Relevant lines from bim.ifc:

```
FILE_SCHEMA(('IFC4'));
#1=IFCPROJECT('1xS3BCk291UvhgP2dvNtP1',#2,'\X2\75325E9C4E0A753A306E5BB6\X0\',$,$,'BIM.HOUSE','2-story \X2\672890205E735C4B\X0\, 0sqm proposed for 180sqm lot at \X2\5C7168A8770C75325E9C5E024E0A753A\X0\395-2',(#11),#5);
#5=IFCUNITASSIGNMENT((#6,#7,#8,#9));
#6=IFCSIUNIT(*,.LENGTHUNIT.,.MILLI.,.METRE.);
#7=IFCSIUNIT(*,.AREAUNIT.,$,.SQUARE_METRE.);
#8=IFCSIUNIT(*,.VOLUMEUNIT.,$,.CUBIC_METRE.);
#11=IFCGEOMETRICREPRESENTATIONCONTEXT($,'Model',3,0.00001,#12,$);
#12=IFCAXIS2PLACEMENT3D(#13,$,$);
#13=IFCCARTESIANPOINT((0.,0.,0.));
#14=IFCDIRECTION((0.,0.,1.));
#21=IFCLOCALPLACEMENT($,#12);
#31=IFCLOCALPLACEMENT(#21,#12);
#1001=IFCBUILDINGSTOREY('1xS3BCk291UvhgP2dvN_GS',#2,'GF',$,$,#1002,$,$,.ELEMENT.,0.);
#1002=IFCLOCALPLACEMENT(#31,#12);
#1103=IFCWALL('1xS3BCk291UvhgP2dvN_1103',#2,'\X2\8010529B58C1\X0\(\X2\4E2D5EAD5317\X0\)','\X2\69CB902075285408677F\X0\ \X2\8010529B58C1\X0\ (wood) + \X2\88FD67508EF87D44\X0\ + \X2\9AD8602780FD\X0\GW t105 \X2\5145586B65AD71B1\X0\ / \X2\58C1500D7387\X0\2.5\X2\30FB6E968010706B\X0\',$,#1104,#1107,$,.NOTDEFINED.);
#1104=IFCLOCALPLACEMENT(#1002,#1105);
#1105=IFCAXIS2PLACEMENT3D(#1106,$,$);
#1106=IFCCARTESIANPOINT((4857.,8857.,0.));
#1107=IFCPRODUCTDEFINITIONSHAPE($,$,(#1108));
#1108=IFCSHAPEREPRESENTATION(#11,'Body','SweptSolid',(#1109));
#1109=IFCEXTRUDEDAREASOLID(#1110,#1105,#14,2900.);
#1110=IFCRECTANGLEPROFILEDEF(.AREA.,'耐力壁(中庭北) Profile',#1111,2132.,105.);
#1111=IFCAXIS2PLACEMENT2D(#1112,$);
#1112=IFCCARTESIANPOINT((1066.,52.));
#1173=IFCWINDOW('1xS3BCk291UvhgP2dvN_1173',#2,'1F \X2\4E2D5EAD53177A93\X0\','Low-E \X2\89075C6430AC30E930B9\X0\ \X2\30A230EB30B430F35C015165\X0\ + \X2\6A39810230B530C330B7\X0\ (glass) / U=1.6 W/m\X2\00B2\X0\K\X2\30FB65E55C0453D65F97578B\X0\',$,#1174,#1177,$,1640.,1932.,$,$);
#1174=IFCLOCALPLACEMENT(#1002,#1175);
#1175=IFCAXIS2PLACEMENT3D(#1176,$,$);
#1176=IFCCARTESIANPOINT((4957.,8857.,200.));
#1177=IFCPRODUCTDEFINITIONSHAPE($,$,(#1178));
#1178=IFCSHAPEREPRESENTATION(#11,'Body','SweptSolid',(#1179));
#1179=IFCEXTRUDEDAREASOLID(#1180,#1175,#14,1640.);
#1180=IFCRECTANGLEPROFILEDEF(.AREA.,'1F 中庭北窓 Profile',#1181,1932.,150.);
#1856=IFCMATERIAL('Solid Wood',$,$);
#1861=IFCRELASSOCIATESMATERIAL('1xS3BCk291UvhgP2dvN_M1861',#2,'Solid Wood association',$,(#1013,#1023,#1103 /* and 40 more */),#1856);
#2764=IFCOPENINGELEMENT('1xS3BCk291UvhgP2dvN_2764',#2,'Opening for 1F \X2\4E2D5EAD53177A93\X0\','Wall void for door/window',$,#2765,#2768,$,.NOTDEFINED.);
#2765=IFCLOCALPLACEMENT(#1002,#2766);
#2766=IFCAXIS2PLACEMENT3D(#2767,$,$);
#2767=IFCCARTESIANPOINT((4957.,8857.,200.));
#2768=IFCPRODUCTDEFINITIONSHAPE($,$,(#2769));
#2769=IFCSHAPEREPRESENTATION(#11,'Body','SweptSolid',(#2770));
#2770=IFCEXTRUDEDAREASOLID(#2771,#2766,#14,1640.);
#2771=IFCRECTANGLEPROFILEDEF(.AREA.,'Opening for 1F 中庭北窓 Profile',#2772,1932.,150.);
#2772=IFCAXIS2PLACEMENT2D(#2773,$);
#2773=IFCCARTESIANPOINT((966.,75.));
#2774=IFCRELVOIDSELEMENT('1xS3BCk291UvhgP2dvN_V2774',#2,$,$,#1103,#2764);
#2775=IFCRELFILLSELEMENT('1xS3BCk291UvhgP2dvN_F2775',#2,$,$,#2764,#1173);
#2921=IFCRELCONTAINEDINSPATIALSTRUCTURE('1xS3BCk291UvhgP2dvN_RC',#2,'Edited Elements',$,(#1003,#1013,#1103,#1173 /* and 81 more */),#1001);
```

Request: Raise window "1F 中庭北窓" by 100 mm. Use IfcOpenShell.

```python
import numpy as np
import ifcopenshell
import ifcopenshell.api.geometry
import ifcopenshell.util.placement
import ifcopenshell.util.unit

model = ifcopenshell.open("bim.ifc")
unit_scale = ifcopenshell.util.unit.calculate_unit_scale(model)

window = model.by_guid("1xS3BCk291UvhgP2dvN_1173")
opening = window.FillsVoids[0].RelatingOpeningElement
dz = 100.0

shift = np.array([0.0, 0.0, dz])
# The window is not placed relative to its opening, so move both.
for product in (opening, window):
    matrix = ifcopenshell.util.placement.get_local_placement(product.ObjectPlacement)
    matrix[:3, 3] += shift
    ifcopenshell.api.geometry.edit_object_placement(model, product=product, matrix=matrix, is_si=False)

print(f"moved by {dz * unit_scale:+.3f} m")

model.write("bim_v2.ifc")
```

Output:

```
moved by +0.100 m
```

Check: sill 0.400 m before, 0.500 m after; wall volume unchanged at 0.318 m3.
